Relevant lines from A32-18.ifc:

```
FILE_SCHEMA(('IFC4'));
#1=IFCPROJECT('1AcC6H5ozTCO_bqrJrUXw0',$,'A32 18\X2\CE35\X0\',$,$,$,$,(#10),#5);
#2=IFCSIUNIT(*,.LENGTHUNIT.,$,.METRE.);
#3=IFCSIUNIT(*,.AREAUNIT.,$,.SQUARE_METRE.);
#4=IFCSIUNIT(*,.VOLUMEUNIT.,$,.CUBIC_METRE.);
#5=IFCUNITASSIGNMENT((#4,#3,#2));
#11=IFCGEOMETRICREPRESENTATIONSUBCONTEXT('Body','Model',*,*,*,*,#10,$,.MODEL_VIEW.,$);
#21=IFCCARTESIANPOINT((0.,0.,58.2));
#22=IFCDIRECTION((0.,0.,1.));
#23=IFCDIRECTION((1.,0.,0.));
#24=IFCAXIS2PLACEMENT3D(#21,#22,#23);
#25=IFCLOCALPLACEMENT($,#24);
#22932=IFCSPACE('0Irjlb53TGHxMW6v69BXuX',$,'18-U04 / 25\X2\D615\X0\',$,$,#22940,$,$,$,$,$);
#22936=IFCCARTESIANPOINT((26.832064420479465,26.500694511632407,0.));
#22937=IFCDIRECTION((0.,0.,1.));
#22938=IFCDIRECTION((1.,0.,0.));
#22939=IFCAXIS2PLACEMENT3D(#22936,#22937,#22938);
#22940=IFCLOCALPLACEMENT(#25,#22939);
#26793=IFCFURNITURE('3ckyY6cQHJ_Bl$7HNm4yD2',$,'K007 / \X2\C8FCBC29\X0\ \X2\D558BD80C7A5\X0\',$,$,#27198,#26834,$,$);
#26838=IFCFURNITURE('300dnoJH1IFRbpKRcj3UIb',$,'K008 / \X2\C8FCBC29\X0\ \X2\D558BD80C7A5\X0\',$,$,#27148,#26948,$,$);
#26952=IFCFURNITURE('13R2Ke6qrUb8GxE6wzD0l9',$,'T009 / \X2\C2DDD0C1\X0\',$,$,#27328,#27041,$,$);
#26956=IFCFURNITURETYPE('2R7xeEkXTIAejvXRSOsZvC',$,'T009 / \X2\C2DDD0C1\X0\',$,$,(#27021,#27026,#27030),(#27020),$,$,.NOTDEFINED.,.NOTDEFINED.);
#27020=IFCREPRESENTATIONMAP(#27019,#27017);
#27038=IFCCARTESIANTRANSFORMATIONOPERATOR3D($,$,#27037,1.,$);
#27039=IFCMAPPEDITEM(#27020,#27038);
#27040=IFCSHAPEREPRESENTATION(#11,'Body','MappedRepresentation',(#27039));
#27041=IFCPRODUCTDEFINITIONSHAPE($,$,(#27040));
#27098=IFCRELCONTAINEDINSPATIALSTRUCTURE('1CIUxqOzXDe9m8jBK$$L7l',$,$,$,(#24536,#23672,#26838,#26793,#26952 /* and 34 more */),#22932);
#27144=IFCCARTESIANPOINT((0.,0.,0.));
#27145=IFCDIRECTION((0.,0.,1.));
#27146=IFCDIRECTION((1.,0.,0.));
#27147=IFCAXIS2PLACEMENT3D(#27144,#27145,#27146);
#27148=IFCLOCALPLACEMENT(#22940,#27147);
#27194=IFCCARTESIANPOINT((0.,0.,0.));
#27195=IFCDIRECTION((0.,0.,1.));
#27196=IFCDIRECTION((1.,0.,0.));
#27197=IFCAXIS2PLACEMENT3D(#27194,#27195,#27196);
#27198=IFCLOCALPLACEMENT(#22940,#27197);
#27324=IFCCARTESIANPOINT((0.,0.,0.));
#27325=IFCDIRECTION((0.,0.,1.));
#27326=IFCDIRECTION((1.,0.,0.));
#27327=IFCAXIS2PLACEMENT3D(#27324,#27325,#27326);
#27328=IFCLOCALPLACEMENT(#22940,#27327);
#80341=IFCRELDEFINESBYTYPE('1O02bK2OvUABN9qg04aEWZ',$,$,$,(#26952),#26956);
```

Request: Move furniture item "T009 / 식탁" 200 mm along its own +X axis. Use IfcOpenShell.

```python
import ifcopenshell
import ifcopenshell.api.geometry
import ifcopenshell.util.placement

model = ifcopenshell.open("A32-18.ifc")

item = model.by_guid("13R2Ke6qrUb8GxE6wzD0l9")
matrix = ifcopenshell.util.placement.get_local_placement(item.ObjectPlacement)
matrix[:3, 3] += matrix[:3, 0] * 0.2
ifcopenshell.api.geometry.edit_object_placement(model, product=item, matrix=matrix, is_si=False)

print(ifcopenshell.util.placement.get_local_placement(item.ObjectPlacement).round(3) + 0.0)

model.write("A32-18_v2.ifc")
```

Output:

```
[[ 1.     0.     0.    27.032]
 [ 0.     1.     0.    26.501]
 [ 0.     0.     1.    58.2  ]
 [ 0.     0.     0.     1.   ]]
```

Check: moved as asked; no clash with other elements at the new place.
